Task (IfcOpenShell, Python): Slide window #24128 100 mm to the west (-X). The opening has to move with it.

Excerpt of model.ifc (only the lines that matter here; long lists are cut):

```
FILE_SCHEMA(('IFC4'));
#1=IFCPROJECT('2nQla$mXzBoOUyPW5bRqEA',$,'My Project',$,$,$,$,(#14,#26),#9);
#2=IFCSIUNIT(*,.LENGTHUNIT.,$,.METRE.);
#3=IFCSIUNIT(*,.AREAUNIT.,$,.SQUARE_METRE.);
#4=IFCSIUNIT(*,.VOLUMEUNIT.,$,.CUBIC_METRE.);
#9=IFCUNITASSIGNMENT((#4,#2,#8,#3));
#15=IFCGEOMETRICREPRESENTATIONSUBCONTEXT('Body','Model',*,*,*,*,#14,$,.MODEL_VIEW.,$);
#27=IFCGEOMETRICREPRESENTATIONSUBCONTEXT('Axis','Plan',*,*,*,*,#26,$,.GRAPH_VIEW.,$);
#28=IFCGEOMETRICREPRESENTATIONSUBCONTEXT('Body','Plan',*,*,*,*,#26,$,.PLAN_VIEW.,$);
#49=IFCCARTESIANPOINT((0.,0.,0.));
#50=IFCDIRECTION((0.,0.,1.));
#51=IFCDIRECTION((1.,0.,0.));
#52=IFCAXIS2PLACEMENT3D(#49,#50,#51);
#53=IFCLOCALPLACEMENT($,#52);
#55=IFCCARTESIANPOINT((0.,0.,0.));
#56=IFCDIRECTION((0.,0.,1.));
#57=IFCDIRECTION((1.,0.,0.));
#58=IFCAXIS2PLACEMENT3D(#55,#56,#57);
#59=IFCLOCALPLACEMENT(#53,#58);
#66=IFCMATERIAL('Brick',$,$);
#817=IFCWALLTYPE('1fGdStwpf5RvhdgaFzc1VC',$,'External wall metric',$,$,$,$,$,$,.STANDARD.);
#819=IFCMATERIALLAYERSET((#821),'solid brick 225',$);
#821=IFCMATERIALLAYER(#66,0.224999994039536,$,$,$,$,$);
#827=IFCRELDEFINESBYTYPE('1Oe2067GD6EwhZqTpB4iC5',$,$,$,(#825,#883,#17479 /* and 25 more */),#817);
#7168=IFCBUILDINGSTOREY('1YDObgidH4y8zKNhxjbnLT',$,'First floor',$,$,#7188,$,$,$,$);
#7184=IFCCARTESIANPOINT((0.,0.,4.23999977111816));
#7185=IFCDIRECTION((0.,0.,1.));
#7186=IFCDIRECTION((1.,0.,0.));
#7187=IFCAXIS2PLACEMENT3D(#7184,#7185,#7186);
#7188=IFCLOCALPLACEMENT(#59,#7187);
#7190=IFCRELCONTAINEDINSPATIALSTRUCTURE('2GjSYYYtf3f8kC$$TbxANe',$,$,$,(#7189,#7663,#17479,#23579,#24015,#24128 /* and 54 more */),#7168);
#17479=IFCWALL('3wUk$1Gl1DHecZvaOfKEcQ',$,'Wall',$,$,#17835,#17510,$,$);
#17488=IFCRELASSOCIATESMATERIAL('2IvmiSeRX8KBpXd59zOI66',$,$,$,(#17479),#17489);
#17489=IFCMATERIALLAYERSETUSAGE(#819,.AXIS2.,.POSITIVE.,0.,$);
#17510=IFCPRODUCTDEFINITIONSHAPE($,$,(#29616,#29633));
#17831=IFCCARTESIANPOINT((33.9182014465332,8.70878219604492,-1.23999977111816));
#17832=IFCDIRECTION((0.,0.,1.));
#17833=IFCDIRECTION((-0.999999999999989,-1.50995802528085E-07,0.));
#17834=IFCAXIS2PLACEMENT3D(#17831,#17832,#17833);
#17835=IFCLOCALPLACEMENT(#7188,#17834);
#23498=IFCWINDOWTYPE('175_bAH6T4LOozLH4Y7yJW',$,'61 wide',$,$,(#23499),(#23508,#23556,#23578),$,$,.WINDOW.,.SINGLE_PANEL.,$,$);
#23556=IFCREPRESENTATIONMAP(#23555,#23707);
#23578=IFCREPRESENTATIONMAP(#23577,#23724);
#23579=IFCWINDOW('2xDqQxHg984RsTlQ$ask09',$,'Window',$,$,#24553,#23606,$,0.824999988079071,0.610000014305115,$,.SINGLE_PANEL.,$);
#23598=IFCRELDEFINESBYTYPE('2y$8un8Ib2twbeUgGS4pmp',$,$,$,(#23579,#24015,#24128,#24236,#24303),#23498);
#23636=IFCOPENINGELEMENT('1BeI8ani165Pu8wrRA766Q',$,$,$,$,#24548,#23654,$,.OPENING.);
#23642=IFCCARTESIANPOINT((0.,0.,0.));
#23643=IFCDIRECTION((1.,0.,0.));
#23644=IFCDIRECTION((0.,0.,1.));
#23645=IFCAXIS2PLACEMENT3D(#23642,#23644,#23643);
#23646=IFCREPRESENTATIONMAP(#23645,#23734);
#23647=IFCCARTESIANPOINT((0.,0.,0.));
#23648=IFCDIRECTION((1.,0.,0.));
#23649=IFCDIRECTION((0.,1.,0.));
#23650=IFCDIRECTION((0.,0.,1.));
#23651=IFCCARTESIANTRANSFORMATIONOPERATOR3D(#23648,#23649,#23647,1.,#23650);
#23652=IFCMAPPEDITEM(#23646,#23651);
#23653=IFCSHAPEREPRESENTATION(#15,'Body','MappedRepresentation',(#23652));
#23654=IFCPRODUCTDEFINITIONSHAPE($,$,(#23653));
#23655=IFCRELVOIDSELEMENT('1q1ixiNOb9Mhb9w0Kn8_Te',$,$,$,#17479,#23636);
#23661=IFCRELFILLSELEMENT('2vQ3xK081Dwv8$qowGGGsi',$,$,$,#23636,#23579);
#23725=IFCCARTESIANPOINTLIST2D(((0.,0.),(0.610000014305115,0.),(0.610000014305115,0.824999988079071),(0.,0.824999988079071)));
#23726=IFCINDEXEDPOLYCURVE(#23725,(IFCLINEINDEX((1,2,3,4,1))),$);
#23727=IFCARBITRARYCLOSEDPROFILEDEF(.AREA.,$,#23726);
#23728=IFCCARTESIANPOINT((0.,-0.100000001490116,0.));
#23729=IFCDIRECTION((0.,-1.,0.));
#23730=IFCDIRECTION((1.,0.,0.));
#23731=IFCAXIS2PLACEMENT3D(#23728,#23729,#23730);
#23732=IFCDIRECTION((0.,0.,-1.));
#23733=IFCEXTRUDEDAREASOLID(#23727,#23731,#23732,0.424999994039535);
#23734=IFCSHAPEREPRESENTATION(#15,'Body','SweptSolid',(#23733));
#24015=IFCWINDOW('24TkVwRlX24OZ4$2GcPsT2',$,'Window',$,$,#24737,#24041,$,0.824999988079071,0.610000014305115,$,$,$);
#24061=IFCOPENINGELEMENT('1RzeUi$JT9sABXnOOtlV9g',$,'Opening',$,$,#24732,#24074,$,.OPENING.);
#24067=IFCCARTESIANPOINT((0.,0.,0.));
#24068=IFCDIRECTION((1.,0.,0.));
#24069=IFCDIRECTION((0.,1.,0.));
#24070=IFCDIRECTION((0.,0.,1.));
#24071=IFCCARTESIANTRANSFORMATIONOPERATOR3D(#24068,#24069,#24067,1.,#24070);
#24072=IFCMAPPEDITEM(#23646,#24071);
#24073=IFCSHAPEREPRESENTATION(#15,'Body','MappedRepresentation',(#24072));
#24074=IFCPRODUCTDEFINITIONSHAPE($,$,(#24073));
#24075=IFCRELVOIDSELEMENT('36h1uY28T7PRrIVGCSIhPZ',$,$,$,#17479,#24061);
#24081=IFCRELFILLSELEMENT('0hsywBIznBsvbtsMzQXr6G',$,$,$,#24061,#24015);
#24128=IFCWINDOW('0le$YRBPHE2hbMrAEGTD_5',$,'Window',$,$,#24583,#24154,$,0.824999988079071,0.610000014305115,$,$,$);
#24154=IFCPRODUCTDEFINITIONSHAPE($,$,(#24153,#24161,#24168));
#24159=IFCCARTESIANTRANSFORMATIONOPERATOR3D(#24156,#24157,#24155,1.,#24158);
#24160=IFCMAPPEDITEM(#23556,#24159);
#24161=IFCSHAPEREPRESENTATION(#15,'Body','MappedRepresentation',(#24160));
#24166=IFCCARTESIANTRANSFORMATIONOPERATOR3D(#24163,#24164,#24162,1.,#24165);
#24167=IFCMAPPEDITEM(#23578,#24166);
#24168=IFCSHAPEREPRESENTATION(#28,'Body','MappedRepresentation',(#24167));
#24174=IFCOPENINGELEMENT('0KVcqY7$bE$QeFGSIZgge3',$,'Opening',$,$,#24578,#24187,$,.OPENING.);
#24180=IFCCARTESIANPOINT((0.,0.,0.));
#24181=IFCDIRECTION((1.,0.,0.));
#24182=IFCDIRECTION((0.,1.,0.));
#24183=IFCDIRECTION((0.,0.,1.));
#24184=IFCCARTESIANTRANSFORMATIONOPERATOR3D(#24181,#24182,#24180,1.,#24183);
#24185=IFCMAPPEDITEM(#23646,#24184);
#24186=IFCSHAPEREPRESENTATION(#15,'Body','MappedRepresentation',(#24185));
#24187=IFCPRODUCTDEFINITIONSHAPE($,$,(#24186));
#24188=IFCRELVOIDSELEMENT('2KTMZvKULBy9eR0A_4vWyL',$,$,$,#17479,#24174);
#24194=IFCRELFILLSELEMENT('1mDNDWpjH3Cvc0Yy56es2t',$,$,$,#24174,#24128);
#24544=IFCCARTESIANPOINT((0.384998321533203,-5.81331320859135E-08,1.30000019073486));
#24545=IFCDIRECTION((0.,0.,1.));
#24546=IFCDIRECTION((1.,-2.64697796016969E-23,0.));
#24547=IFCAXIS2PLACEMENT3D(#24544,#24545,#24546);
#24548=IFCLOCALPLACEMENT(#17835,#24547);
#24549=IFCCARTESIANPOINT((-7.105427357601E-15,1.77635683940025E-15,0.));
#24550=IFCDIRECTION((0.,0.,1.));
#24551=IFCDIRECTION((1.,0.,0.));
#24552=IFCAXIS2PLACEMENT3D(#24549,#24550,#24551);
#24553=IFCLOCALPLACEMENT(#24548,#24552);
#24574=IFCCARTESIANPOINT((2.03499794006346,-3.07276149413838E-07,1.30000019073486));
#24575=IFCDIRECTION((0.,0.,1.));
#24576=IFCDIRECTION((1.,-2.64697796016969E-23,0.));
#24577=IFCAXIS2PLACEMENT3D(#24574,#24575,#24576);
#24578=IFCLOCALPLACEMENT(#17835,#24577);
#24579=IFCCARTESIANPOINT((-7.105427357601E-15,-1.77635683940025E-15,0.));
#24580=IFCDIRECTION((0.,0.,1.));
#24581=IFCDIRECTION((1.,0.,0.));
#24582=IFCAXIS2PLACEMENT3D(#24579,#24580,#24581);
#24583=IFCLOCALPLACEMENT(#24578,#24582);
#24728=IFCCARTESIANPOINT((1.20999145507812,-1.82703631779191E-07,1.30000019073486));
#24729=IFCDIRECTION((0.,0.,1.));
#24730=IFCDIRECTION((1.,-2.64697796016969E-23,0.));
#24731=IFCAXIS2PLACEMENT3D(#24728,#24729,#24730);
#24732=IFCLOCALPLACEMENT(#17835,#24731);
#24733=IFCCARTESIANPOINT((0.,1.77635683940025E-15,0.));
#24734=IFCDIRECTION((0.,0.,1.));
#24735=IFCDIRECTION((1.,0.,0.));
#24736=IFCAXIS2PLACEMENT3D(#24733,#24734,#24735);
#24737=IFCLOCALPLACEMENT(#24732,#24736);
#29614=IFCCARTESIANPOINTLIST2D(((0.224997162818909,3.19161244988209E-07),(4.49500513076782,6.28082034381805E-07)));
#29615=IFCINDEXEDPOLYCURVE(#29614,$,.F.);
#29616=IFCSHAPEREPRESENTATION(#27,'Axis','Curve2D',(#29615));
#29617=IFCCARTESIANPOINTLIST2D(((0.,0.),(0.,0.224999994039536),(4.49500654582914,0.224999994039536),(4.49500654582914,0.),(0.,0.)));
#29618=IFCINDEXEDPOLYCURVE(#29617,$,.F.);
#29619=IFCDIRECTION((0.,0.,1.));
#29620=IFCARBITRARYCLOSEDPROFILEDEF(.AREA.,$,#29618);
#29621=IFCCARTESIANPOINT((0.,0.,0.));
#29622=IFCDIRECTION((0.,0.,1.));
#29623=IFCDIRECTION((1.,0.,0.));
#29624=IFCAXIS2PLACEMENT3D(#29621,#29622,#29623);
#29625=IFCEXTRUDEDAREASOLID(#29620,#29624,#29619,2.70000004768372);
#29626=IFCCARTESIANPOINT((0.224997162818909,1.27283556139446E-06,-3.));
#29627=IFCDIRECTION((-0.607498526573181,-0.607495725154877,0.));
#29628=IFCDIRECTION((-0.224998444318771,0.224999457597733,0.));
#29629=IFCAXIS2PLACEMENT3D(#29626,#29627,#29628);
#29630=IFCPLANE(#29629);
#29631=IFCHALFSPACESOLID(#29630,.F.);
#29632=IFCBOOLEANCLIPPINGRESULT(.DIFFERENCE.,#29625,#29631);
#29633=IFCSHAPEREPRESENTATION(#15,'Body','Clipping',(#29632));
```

```python
import ifcopenshell
import ifcopenshell.api.geometry
import ifcopenshell.util.placement
import ifcopenshell.util.unit

model = ifcopenshell.open("model.ifc")
unit_scale = ifcopenshell.util.unit.calculate_unit_scale(model)

window = model.by_guid("0le$YRBPHE2hbMrAEGTD_5")
opening = window.FillsVoids[0].RelatingOpeningElement
wall = opening.VoidsElements[0].RelatingBuildingElement

wall_matrix = ifcopenshell.util.placement.get_local_placement(wall.ObjectPlacement)
shift = wall_matrix[:3, 0] * 0.1 / unit_scale
before = ifcopenshell.util.placement.get_local_placement(window.ObjectPlacement)[:3, 3].copy()

# The window is placed relative to its opening, so it follows when the opening moves.
matrix = ifcopenshell.util.placement.get_local_placement(opening.ObjectPlacement)
matrix[:3, 3] += shift
ifcopenshell.api.geometry.edit_object_placement(
    model, product=opening, matrix=matrix, is_si=False, should_transform_children=True
)

after = ifcopenshell.util.placement.get_local_placement(window.ObjectPlacement)[:3, 3]
print("window moved by", (after - before).round(3) + 0.0)

model.write("model_updated.ifc")
```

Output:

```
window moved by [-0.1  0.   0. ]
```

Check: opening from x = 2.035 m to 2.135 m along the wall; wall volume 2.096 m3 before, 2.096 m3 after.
